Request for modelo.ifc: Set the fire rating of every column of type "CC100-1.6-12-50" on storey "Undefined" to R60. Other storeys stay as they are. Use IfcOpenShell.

First a look at what the model holds.

```python
import ifcopenshell
import ifcopenshell.util.element

model = ifcopenshell.open("modelo.ifc")
print(model.schema)
storey = next(s for s in model.by_type("IfcBuildingStorey") if s.Name == "Undefined")
columns = [e for e in ifcopenshell.util.element.get_decomposition(storey) if e.is_a("IfcColumn")]
seen = {}
for e in columns:
    element_type = ifcopenshell.util.element.get_type(e)
    key = (element_type.Name if element_type != e and element_type else None, ifcopenshell.util.element.get_pset(e, "Pset_ColumnCommon", "FireRating"))
    seen[key] = seen.get(key, 0) + 1
for (name, value), count in sorted(seen.items(), key=str):
    print(count, "x", name, "|", value)
```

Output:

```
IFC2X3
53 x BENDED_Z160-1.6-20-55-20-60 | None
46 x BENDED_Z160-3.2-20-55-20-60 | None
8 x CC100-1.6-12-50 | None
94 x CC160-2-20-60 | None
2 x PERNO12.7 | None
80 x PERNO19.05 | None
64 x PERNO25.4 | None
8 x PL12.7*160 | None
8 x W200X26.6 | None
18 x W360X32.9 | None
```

```python
import ifcopenshell
import ifcopenshell.api.pset
import ifcopenshell.util.element

model = ifcopenshell.open("modelo.ifc")

storey = next(s for s in model.by_type("IfcBuildingStorey") if s.Name == "Undefined")
columns = [e for e in ifcopenshell.util.element.get_decomposition(storey) if e.is_a("IfcColumn")]

count = 0
for e in columns:
    element_type = ifcopenshell.util.element.get_type(e)
    if element_type in (None, e) or element_type.Name != "CC100-1.6-12-50":
        continue
    found = ifcopenshell.util.element.get_pset(e, "Pset_ColumnCommon", should_inherit=False)
    if found:
        pset = model.by_id(found["id"])
        if len(ifcopenshell.util.element.get_elements_by_pset(pset)) > 1:
            pset = ifcopenshell.api.pset.unshare_pset(model, products=[e], pset=pset)[0]
    else:
        pset = ifcopenshell.api.pset.add_pset(model, product=e, name="Pset_ColumnCommon")
    ifcopenshell.api.pset.edit_pset(model, pset=pset, properties={"FireRating": "R60"})
    count += 1

print(count, "columns updated")

model.write("modelo_edited.ifc")
```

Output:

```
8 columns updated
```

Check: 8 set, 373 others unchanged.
